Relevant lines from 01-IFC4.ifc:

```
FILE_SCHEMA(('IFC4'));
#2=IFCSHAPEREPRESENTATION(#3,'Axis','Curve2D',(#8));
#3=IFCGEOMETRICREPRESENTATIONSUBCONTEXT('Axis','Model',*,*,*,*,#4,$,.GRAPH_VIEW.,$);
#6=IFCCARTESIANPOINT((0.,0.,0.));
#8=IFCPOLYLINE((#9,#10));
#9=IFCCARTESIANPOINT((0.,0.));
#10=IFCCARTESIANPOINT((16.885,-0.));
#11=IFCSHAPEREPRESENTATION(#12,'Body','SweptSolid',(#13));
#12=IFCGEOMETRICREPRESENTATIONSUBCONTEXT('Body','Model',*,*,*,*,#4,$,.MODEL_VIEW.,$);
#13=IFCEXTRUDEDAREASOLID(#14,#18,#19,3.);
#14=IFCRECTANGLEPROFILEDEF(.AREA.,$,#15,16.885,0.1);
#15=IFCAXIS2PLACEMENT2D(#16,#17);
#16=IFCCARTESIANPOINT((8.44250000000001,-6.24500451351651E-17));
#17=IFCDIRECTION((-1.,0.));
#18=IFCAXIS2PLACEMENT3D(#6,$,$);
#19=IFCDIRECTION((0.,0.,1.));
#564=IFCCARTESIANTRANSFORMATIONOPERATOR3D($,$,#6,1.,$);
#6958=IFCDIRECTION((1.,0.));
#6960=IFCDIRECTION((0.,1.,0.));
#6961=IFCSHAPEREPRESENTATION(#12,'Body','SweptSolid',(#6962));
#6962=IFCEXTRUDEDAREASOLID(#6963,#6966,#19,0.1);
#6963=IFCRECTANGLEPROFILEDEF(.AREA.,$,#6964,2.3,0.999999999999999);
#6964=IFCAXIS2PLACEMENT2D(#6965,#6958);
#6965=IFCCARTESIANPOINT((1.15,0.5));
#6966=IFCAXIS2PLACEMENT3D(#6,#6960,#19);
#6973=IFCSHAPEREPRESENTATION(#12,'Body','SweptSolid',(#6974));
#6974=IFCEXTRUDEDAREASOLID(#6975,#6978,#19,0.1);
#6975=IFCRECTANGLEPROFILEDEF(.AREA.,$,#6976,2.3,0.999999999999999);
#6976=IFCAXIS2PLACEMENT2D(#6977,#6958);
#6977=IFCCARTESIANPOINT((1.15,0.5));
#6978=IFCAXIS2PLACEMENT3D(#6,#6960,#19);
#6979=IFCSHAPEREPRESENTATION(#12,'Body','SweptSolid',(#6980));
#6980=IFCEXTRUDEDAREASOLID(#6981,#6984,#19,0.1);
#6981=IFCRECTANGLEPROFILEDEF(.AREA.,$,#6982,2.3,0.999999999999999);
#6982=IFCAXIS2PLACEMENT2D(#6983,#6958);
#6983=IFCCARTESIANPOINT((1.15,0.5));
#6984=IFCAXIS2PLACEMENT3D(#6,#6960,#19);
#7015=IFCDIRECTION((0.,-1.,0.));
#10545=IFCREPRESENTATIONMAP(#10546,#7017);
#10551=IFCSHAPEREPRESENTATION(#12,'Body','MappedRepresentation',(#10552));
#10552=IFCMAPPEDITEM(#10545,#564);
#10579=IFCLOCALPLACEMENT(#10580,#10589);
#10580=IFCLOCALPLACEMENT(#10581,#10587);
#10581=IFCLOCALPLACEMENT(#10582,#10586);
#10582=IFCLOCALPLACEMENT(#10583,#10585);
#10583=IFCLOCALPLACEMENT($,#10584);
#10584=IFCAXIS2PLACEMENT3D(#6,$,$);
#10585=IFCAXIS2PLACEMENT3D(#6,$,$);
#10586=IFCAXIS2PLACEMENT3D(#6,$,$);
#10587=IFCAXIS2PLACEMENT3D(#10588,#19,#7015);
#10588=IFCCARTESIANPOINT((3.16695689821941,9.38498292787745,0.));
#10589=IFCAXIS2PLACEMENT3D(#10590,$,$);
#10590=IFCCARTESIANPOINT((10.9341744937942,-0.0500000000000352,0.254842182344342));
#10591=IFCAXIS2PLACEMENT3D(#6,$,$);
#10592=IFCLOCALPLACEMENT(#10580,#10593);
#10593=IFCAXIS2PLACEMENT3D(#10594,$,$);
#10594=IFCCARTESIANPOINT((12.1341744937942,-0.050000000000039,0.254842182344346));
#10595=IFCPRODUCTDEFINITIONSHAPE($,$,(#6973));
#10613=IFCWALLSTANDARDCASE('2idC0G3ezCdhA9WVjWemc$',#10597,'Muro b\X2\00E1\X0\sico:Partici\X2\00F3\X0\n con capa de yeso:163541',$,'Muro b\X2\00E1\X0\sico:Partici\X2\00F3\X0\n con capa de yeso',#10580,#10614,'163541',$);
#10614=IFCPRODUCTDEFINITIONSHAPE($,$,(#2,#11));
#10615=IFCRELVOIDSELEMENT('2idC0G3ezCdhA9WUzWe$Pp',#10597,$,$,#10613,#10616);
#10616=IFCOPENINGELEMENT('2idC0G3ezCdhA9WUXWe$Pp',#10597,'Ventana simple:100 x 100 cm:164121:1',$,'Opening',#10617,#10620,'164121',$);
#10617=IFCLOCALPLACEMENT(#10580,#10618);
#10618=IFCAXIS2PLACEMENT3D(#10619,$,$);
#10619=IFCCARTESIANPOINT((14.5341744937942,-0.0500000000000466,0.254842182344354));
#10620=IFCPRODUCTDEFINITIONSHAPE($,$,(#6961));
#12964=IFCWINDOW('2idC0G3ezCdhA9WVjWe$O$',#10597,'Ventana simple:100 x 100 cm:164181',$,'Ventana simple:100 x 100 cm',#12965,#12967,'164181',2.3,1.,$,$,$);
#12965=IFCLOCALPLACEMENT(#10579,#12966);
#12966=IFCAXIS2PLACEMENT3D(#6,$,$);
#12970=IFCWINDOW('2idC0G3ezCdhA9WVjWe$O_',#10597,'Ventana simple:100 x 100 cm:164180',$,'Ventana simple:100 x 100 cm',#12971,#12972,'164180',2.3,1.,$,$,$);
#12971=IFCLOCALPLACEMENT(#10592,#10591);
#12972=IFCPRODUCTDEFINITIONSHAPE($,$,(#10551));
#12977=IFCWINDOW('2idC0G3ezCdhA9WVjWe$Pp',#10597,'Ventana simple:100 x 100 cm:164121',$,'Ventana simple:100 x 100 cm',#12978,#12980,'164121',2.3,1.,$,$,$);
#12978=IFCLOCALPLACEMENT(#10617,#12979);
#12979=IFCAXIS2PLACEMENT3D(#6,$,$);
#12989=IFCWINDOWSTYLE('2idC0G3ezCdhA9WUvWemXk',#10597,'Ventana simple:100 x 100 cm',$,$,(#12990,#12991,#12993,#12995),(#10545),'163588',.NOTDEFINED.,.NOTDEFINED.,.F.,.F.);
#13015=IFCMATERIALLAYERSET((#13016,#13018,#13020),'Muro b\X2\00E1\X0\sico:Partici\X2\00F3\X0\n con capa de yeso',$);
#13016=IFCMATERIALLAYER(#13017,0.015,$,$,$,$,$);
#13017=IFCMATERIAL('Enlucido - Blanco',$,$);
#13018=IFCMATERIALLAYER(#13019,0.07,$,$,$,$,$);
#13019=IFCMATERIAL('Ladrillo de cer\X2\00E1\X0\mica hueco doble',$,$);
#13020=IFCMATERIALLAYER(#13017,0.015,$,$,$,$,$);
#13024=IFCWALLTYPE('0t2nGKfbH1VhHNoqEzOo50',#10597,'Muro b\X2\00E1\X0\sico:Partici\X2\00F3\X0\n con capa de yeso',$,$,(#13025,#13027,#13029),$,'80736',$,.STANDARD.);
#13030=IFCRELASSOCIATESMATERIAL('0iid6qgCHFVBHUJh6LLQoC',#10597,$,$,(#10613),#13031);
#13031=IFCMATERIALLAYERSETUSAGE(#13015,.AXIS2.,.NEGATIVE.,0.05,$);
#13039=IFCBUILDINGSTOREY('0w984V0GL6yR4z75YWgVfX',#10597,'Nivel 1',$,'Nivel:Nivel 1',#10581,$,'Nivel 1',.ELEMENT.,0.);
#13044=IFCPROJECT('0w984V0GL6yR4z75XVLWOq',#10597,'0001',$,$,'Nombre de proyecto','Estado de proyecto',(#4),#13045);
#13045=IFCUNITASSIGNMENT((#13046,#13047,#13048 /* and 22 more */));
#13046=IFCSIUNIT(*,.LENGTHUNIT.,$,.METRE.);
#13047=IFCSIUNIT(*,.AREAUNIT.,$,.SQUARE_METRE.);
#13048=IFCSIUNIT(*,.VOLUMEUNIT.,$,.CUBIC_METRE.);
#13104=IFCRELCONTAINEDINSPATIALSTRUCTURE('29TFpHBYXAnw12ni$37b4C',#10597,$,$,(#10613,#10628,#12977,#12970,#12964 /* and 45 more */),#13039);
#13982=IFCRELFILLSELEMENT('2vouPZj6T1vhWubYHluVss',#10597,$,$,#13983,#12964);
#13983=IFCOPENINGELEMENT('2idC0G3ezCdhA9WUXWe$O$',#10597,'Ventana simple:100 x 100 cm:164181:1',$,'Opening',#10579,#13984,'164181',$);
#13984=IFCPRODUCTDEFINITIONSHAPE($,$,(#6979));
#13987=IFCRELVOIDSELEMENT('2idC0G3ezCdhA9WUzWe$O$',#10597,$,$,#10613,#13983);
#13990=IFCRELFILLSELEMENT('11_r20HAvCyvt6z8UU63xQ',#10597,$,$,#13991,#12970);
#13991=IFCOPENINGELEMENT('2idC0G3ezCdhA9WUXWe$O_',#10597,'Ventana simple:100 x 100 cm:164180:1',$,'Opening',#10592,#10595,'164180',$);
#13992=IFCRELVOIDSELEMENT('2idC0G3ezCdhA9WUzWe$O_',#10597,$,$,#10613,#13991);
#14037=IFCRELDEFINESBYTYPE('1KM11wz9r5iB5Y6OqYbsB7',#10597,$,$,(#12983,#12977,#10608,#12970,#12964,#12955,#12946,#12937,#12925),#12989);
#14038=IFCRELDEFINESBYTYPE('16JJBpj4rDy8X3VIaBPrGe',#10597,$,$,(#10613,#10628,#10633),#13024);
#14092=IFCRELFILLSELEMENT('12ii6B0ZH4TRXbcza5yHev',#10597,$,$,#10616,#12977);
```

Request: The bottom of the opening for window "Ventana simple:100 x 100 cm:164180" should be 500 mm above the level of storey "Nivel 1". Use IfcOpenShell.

```python
import numpy as np
import ifcopenshell
import ifcopenshell.api.geometry
import ifcopenshell.geom
import ifcopenshell.util.element
import ifcopenshell.util.placement
import ifcopenshell.util.shape
import ifcopenshell.util.unit

model = ifcopenshell.open("01-IFC4.ifc")
unit_scale = ifcopenshell.util.unit.calculate_unit_scale(model)

window = model.by_guid("2idC0G3ezCdhA9WVjWe$O_")
opening = window.FillsVoids[0].RelatingOpeningElement
storey = ifcopenshell.util.element.get_container(window, ifc_class="IfcBuildingStorey")
level = ifcopenshell.util.placement.get_local_placement(storey.ObjectPlacement)[2, 3]

# The opening's origin need not be at the sill, so measure its lowest point.
shape = ifcopenshell.geom.create_shape(ifcopenshell.geom.settings(), opening)
bottom = ifcopenshell.util.shape.get_shape_bottom_elevation(shape, shape.geometry) / unit_scale
dz = level + 0.5 / unit_scale - bottom

shift = np.array([0.0, 0.0, dz])
# The window is placed relative to its opening, so it follows when the opening moves.
matrix = ifcopenshell.util.placement.get_local_placement(opening.ObjectPlacement)
matrix[:3, 3] += shift
ifcopenshell.api.geometry.edit_object_placement(
    model, product=opening, matrix=matrix, is_si=False, should_transform_children=True
)

print(f"moved by {dz * unit_scale:+.3f} m")

model.write("01-IFC4_rev.ifc")
```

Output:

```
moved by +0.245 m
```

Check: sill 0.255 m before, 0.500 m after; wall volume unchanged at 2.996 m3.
